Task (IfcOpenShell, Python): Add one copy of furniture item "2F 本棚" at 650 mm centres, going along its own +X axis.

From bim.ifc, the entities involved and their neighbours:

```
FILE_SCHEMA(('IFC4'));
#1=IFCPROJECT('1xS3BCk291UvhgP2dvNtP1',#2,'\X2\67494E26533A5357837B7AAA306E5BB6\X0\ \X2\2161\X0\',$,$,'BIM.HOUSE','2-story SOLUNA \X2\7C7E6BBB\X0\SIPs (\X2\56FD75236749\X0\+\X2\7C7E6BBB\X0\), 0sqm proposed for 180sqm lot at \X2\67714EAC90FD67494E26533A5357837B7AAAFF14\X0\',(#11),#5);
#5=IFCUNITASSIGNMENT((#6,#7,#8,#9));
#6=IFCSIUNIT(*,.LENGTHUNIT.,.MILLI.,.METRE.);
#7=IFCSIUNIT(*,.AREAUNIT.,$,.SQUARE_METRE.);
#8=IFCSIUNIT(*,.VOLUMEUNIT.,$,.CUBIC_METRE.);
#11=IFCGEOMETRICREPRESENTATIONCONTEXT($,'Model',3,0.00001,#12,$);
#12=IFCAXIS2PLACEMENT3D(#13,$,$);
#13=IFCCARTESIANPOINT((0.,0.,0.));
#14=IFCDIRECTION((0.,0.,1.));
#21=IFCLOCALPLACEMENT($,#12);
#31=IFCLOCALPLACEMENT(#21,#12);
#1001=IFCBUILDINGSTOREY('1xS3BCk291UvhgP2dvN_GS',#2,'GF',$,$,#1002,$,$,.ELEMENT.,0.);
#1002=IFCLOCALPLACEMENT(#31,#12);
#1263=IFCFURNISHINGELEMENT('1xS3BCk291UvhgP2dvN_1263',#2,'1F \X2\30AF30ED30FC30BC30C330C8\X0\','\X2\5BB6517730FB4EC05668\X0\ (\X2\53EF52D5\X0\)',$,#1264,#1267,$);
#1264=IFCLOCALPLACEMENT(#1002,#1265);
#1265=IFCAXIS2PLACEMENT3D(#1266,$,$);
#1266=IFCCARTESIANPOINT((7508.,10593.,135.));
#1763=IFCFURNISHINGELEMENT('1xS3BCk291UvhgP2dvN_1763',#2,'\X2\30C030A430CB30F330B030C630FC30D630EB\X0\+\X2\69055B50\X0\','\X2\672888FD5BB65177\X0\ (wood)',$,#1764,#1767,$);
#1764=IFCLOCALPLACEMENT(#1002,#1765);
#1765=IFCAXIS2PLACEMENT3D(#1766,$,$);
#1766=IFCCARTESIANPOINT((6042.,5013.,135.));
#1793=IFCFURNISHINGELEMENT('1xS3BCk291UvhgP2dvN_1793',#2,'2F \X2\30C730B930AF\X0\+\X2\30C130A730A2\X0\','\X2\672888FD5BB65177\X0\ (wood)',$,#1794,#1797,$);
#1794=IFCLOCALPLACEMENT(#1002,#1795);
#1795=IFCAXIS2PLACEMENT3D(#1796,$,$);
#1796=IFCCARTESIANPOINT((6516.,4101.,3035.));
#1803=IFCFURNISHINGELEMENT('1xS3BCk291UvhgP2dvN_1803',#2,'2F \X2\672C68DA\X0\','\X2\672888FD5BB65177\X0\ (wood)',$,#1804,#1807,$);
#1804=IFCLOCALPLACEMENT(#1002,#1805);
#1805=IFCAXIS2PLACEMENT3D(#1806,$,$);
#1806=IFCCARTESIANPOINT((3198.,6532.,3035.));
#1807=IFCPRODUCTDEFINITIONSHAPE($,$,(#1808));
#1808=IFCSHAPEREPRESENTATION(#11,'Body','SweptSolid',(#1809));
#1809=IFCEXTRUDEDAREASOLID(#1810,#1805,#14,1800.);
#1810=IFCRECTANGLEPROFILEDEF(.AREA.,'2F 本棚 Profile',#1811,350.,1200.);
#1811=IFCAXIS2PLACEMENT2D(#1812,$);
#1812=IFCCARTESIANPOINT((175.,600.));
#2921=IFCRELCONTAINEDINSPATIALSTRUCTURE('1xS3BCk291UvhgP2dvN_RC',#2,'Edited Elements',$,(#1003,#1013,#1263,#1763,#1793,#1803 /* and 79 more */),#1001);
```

```python
import ifcopenshell
import ifcopenshell.api.geometry
import ifcopenshell.api.root
import ifcopenshell.util.element
import ifcopenshell.util.placement
import ifcopenshell.util.unit

model = ifcopenshell.open("bim.ifc")
unit_scale = ifcopenshell.util.unit.calculate_unit_scale(model)


def reuse_history(source, copy):
    """copy_class also copies each property set's owner history, people and application; keep the originals."""
    for rel in copy.IsDefinedBy:
        if rel.is_a("IfcRelDefinesByProperties") and (history := rel.RelatingPropertyDefinition.OwnerHistory):
            rel.RelatingPropertyDefinition.OwnerHistory = source.OwnerHistory
            ifcopenshell.util.element.remove_deep2(model, history)


source = model.by_guid("1xS3BCk291UvhgP2dvN_1803")
base = ifcopenshell.util.placement.get_local_placement(source.ObjectPlacement)
step = base[:3, 0] * 0.65 / unit_scale

for i in range(1, 2):
    copy = ifcopenshell.api.root.copy_class(model, product=source)
    copy.Representation = ifcopenshell.util.element.copy_deep(
        model, source.Representation, exclude=["IfcGeometricRepresentationContext", "IfcRepresentationMap"]
    )
    reuse_history(source, copy)
    matrix = base.copy()
    matrix[:3, 3] += i * step
    print("added at", matrix[:3, 3].round(3) + 0.0)
    ifcopenshell.api.geometry.edit_object_placement(model, product=copy, matrix=matrix, is_si=False)

model.write("bim_edited.ifc")
```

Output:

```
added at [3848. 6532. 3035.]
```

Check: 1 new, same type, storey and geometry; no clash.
